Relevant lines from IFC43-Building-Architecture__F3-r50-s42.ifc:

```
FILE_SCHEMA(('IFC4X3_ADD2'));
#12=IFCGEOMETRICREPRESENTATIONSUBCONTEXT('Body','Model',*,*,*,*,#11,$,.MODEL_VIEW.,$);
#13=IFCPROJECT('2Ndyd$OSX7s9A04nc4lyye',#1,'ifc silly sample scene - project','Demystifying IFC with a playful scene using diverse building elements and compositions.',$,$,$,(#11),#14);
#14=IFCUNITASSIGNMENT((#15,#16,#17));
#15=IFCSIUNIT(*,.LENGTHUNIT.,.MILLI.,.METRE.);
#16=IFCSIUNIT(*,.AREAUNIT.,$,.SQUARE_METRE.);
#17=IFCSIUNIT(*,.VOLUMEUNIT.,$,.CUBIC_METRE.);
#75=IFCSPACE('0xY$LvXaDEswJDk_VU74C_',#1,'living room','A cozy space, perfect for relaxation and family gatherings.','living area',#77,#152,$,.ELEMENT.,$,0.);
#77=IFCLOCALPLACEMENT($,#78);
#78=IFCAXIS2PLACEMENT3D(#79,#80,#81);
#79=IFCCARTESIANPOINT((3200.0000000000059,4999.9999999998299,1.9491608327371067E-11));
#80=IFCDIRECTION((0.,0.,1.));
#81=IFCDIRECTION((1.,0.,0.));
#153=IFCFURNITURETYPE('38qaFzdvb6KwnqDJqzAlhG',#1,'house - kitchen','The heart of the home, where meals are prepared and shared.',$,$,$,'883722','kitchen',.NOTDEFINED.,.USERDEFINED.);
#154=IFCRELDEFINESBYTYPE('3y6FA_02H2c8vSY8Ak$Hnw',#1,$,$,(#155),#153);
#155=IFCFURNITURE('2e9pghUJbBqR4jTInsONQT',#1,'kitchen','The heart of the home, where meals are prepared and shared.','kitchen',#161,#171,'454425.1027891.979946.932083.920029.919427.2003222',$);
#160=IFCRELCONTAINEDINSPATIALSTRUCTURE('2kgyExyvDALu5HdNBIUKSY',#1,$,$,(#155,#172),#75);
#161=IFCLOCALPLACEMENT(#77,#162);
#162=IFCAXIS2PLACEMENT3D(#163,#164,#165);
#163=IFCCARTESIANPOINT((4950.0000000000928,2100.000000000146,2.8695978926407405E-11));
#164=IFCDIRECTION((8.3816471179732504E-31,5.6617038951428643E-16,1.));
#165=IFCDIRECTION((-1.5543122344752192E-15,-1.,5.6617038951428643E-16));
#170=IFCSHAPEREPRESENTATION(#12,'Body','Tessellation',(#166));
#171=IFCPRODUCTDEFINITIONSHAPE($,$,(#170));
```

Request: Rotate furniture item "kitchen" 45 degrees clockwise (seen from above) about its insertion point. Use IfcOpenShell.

```python
import ifcopenshell
import ifcopenshell.api.geometry
import ifcopenshell.util.placement

model = ifcopenshell.open("IFC43-Building-Architecture__F3-r50-s42.ifc")

item = model.by_guid("2e9pghUJbBqR4jTInsONQT")
matrix = ifcopenshell.util.placement.get_local_placement(item.ObjectPlacement)
matrix = matrix @ ifcopenshell.util.placement.rotation(-45, "Z")
ifcopenshell.api.geometry.edit_object_placement(model, product=item, matrix=matrix, is_si=False)

print(ifcopenshell.util.placement.get_local_placement(item.ObjectPlacement).round(3) + 0.0)

model.write("IFC43-Building-Architecture__F3-r50-s42_rev.ifc")
```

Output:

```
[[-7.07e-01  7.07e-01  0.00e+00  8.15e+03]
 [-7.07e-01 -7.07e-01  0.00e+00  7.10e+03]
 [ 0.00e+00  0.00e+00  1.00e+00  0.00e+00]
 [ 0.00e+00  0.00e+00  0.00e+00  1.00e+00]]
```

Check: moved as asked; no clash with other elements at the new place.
